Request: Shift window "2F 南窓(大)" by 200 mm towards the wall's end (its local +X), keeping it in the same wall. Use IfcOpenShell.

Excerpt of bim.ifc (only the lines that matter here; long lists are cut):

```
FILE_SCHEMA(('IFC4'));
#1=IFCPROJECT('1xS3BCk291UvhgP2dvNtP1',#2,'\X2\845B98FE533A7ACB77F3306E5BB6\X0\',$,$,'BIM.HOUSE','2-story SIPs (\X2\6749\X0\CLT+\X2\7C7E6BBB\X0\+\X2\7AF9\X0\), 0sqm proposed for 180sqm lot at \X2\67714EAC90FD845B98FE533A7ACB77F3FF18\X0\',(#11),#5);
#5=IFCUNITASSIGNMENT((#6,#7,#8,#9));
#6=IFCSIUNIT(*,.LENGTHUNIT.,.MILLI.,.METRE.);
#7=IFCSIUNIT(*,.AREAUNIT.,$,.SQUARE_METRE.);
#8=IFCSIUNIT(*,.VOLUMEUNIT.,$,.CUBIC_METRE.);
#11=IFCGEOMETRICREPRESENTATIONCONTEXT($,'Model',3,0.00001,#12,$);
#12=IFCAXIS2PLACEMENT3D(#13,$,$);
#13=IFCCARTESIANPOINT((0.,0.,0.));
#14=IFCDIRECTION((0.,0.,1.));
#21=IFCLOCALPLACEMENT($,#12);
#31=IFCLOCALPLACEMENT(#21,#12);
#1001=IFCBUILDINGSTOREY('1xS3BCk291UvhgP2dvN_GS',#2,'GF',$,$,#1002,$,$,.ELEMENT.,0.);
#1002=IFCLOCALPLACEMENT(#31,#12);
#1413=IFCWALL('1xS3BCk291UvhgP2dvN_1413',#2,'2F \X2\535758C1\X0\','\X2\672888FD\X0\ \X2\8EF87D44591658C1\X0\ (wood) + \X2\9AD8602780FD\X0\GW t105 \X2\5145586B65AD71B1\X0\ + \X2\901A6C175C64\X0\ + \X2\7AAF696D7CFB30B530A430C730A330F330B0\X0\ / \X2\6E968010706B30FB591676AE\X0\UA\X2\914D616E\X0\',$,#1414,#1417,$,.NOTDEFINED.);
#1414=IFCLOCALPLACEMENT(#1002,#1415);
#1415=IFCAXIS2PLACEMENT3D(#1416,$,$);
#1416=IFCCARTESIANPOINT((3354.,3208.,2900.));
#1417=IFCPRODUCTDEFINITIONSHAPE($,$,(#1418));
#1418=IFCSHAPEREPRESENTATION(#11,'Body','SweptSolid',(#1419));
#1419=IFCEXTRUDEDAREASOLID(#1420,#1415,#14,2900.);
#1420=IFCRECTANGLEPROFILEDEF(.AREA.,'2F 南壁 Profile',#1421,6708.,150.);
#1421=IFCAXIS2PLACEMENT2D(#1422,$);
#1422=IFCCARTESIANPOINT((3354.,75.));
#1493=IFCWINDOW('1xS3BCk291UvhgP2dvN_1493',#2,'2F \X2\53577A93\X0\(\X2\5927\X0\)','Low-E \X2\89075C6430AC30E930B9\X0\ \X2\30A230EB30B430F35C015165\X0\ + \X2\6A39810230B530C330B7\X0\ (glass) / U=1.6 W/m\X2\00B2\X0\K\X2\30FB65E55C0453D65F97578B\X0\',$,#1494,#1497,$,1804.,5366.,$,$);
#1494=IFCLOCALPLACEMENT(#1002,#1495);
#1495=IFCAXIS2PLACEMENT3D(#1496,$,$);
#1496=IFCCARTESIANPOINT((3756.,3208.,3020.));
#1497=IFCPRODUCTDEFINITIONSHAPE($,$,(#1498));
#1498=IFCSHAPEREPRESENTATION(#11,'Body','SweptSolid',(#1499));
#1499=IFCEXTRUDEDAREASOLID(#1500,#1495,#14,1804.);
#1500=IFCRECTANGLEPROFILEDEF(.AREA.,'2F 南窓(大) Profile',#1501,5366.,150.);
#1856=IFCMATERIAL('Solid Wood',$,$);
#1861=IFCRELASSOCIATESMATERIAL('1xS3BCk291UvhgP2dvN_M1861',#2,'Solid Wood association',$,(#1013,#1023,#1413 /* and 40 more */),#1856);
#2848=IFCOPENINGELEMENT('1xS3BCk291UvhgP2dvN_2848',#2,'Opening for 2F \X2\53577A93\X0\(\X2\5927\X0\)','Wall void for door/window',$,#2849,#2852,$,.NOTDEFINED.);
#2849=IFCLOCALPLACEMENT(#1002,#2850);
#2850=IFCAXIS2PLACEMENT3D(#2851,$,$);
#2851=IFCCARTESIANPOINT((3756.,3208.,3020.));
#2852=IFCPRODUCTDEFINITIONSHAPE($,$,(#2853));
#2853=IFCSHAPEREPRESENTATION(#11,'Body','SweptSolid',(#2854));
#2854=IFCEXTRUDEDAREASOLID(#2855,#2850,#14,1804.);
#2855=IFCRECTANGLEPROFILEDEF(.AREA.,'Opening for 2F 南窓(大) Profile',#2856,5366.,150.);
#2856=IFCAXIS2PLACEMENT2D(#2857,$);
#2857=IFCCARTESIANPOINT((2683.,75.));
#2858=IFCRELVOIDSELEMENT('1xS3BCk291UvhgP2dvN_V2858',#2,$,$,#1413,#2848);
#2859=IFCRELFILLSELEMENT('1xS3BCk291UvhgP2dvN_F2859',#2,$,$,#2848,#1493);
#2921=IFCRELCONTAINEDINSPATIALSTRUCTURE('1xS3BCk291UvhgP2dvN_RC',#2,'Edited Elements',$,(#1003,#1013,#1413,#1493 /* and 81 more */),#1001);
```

```python
import ifcopenshell
import ifcopenshell.api.geometry
import ifcopenshell.util.placement
import ifcopenshell.util.unit

model = ifcopenshell.open("bim.ifc")
unit_scale = ifcopenshell.util.unit.calculate_unit_scale(model)

window = model.by_guid("1xS3BCk291UvhgP2dvN_1493")
opening = window.FillsVoids[0].RelatingOpeningElement
wall = opening.VoidsElements[0].RelatingBuildingElement

wall_matrix = ifcopenshell.util.placement.get_local_placement(wall.ObjectPlacement)
shift = wall_matrix[:3, 0] * 0.2 / unit_scale
before = ifcopenshell.util.placement.get_local_placement(window.ObjectPlacement)[:3, 3].copy()

# The window is not placed relative to its opening, so move both.
for product in (opening, window):
    matrix = ifcopenshell.util.placement.get_local_placement(product.ObjectPlacement)
    matrix[:3, 3] += shift
    ifcopenshell.api.geometry.edit_object_placement(model, product=product, matrix=matrix, is_si=False)

after = ifcopenshell.util.placement.get_local_placement(window.ObjectPlacement)[:3, 3]
print("window moved by", (after - before).round(3) + 0.0)

model.write("bim-out.ifc")
```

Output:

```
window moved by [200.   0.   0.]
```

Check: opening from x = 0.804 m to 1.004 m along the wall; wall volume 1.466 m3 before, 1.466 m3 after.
